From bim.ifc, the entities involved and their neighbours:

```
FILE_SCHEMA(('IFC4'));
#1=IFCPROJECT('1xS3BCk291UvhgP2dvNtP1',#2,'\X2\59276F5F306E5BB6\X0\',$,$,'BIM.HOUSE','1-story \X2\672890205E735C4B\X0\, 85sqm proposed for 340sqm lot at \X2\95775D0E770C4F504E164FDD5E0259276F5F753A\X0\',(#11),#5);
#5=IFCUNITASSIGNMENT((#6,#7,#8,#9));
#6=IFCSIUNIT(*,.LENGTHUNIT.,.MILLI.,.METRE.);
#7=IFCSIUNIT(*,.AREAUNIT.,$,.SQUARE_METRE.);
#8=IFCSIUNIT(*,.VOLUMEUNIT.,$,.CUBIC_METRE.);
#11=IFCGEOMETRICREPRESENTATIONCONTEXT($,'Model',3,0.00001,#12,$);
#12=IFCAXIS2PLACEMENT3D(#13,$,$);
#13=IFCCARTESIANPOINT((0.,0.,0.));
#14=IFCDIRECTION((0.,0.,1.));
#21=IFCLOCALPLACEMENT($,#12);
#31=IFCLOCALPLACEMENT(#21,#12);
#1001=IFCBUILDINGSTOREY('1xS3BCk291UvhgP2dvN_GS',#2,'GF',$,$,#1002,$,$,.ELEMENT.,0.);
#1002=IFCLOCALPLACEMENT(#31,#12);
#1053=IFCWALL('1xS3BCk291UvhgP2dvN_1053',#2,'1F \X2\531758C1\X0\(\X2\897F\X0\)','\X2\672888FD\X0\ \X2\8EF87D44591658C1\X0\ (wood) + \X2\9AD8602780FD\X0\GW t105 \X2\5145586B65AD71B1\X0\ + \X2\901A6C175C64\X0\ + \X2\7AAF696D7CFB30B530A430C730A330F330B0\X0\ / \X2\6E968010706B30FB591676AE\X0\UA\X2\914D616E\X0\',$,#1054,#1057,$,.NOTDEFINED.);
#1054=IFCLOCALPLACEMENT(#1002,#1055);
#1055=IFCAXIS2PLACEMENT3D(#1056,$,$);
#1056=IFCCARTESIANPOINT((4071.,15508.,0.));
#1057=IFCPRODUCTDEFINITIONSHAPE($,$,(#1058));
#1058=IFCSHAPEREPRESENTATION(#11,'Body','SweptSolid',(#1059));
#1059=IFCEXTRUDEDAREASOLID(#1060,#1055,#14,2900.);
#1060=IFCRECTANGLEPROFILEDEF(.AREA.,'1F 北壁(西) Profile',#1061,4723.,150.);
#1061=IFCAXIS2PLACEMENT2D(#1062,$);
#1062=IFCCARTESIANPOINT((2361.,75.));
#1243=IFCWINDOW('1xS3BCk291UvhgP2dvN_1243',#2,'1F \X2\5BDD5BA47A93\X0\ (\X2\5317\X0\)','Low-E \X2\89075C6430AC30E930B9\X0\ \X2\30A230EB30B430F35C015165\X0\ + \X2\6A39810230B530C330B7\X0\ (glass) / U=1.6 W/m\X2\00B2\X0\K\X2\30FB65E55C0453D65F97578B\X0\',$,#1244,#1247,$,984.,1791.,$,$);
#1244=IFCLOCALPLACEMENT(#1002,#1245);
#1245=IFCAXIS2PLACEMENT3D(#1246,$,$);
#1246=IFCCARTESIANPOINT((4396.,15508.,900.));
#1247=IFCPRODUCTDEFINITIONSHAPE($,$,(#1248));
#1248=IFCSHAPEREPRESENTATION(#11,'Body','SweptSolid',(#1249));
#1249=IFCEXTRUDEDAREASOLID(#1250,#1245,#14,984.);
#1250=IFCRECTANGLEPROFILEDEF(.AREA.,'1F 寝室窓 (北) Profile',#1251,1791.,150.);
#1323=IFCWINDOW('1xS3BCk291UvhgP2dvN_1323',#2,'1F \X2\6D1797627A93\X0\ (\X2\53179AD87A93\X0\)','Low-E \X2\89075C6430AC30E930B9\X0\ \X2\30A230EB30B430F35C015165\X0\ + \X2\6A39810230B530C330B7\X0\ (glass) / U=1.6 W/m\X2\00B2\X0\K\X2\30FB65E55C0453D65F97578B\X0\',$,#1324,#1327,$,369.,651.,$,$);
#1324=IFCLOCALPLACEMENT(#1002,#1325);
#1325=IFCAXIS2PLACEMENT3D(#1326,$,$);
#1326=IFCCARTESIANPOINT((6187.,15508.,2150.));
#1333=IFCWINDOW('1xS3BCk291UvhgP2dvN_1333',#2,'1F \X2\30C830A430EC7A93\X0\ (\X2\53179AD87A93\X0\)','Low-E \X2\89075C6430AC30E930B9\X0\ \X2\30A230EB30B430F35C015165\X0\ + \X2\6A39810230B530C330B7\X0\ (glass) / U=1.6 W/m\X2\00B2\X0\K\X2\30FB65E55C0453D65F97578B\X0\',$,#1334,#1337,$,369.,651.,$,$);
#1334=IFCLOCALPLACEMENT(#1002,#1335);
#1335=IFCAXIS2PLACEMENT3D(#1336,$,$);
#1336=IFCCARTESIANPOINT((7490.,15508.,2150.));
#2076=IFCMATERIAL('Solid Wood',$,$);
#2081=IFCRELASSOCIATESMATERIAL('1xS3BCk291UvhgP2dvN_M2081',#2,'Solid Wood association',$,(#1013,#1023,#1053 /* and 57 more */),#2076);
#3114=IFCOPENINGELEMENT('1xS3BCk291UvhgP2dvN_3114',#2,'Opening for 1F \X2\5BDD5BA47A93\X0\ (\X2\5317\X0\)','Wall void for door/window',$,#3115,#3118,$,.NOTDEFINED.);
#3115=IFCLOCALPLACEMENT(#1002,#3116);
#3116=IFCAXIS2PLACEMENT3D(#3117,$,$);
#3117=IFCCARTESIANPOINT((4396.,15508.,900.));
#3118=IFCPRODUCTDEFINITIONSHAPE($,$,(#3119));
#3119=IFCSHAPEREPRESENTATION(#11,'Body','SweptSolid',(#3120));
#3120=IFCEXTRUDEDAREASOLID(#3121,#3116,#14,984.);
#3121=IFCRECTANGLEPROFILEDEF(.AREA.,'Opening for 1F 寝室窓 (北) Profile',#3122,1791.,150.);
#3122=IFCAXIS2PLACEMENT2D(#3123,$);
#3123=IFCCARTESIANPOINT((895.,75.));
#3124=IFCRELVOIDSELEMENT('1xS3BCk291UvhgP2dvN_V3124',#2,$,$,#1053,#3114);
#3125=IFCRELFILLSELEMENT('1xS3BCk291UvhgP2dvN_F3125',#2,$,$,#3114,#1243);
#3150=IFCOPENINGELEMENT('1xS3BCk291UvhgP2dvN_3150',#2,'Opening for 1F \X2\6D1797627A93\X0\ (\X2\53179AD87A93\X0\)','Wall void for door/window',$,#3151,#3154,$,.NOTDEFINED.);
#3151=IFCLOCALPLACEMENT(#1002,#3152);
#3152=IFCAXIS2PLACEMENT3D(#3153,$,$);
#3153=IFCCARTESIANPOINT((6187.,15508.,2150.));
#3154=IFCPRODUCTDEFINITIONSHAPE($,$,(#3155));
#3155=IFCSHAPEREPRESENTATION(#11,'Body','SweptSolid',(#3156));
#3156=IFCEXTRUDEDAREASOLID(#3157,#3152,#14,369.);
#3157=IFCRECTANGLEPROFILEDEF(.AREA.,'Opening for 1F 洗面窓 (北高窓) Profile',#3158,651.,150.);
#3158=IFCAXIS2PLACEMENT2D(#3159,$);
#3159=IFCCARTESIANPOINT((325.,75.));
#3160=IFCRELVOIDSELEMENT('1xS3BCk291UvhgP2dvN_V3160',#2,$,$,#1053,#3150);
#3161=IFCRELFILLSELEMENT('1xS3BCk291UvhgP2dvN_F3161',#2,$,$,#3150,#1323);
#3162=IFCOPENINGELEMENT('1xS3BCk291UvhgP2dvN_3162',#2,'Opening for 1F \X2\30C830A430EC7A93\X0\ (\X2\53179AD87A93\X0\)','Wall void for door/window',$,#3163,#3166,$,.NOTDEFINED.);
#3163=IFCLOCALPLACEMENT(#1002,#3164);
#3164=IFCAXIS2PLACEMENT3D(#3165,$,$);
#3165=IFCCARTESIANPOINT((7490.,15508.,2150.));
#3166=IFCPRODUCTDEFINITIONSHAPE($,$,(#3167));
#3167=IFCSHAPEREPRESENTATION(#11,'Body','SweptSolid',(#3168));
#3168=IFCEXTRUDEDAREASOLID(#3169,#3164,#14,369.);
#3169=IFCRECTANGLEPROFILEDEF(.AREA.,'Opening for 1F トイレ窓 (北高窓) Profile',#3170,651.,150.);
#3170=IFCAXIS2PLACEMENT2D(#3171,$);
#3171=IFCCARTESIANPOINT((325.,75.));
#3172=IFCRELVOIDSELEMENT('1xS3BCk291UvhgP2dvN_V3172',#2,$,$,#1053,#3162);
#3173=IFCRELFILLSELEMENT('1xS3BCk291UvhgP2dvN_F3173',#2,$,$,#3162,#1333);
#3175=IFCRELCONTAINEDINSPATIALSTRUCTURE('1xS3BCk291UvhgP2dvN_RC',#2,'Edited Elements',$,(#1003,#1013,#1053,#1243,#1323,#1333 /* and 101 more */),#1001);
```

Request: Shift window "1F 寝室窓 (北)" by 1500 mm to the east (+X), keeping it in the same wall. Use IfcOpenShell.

```python
import ifcopenshell
import ifcopenshell.api.geometry
import ifcopenshell.util.placement
import ifcopenshell.util.unit

model = ifcopenshell.open("bim.ifc")
unit_scale = ifcopenshell.util.unit.calculate_unit_scale(model)

window = model.by_guid("1xS3BCk291UvhgP2dvN_1243")
opening = window.FillsVoids[0].RelatingOpeningElement
wall = opening.VoidsElements[0].RelatingBuildingElement

wall_matrix = ifcopenshell.util.placement.get_local_placement(wall.ObjectPlacement)
shift = wall_matrix[:3, 0] * 1.5 / unit_scale
before = ifcopenshell.util.placement.get_local_placement(window.ObjectPlacement)[:3, 3].copy()

# The window is not placed relative to its opening, so move both.
for product in (opening, window):
    matrix = ifcopenshell.util.placement.get_local_placement(product.ObjectPlacement)
    matrix[:3, 3] += shift
    ifcopenshell.api.geometry.edit_object_placement(model, product=product, matrix=matrix, is_si=False)

after = ifcopenshell.util.placement.get_local_placement(window.ObjectPlacement)[:3, 3]
print("window moved by", (after - before).round(3) + 0.0)

model.write("bim_edited.ifc")
```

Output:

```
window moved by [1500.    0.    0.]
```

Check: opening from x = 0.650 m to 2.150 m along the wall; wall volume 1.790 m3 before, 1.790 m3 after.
